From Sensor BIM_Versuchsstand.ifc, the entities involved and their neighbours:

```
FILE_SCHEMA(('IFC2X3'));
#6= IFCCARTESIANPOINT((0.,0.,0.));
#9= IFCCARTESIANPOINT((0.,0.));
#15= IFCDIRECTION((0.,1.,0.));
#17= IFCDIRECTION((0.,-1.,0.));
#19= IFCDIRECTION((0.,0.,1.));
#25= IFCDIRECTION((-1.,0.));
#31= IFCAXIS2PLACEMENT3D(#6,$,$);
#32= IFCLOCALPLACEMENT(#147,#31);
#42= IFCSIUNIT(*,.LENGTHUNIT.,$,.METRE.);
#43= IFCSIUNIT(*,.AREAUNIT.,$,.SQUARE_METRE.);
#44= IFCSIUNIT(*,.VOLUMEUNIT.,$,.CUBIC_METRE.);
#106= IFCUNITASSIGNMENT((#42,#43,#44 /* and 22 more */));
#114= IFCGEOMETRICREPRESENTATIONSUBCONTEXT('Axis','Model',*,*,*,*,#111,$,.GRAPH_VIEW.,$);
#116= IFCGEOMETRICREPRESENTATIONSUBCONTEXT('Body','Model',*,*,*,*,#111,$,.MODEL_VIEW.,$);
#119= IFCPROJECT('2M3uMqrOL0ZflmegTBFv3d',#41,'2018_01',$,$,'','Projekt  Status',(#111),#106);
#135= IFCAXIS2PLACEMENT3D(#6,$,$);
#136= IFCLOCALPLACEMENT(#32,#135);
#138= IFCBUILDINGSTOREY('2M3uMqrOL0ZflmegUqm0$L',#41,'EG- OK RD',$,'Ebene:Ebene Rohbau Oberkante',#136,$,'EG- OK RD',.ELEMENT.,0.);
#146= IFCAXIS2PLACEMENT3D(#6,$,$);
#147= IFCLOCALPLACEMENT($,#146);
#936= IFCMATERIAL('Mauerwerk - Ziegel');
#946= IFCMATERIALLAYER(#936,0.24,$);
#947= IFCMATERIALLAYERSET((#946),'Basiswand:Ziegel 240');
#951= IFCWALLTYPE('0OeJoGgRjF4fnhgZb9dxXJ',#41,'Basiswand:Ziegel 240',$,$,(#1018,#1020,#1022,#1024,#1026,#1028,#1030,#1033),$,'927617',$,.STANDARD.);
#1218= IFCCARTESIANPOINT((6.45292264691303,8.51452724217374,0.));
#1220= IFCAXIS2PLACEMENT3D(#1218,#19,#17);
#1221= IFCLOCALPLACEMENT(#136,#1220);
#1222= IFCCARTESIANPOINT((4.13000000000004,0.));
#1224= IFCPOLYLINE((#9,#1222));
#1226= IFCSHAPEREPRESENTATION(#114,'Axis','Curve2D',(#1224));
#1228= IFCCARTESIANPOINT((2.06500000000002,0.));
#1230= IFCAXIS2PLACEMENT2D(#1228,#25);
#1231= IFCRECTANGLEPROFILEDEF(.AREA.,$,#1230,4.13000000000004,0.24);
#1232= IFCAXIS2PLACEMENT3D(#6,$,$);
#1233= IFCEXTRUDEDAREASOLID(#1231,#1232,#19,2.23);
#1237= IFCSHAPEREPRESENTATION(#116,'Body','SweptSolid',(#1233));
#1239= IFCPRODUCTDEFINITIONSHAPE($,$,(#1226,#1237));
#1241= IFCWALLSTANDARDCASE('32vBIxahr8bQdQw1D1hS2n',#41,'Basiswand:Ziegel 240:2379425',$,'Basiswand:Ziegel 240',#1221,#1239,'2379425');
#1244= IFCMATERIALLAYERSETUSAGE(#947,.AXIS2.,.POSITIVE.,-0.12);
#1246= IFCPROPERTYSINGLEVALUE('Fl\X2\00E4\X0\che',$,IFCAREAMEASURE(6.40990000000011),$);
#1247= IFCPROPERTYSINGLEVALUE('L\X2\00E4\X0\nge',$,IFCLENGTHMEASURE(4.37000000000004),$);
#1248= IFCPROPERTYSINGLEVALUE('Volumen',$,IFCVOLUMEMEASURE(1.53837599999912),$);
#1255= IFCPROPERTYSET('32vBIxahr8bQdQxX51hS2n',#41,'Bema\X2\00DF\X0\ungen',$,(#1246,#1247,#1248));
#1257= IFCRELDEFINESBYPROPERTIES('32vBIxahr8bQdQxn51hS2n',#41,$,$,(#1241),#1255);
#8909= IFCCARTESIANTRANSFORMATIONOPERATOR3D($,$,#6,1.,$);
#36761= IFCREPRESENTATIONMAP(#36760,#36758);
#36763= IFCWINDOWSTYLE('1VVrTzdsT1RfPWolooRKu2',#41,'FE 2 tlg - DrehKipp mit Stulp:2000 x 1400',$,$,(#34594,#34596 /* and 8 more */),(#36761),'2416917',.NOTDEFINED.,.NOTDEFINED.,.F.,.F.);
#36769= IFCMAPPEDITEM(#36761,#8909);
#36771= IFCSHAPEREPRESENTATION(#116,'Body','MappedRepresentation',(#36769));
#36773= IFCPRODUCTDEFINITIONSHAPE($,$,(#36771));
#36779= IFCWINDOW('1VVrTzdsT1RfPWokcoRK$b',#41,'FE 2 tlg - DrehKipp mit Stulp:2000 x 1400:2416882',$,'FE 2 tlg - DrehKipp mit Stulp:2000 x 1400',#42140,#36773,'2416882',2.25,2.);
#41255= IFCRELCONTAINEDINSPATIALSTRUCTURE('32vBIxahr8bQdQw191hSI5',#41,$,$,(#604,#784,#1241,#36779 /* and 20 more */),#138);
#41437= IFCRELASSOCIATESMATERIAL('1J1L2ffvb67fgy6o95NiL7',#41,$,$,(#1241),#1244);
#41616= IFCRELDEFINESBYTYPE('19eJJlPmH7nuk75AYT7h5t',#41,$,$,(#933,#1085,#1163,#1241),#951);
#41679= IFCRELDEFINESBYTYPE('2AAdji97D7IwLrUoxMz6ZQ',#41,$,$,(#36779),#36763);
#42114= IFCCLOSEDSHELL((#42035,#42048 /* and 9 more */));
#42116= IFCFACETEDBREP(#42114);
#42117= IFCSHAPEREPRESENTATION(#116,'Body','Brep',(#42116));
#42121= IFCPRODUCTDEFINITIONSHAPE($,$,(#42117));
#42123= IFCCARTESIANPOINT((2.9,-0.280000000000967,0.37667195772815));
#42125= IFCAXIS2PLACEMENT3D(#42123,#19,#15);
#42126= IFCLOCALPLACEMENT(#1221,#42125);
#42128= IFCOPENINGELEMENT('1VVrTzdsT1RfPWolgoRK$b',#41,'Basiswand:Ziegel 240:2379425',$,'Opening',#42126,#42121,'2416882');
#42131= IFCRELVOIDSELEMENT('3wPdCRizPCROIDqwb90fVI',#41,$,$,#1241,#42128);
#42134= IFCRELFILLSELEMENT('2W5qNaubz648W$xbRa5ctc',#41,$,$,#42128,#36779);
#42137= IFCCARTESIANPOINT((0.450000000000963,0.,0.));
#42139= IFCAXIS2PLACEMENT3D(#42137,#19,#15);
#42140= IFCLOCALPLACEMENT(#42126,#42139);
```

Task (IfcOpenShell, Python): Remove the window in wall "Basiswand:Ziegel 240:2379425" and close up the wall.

```python
import ifcopenshell
import ifcopenshell.api.feature
import ifcopenshell.api.pset
import ifcopenshell.api.root
import ifcopenshell.geom
import ifcopenshell.util.element
import ifcopenshell.util.shape
import ifcopenshell.util.unit

model = ifcopenshell.open("Sensor BIM_Versuchsstand.ifc")
area_scale = ifcopenshell.util.unit.calculate_unit_scale(model, "AREAUNIT")
volume_scale = ifcopenshell.util.unit.calculate_unit_scale(model, "VOLUMEUNIT")
settings = ifcopenshell.geom.settings()


def volume(element):
    """Net volume in cubic metres, openings subtracted."""
    shape = ifcopenshell.geom.create_shape(settings, element)
    return ifcopenshell.util.shape.get_volume(shape.geometry)


window = model.by_id(36779)
opening = window.FillsVoids[0].RelatingOpeningElement
wall = opening.VoidsElements[0].RelatingBuildingElement
before = volume(wall)

ifcopenshell.api.root.remove_product(model, product=window)
ifcopenshell.api.feature.remove_feature(model, feature=opening)

after = volume(wall)
thickness = 0.24  # wall thickness in metres

# Update the wall's stored quantities.
pset = model.by_id(ifcopenshell.util.element.get_pset(wall, "Bemaßungen", should_inherit=False)["id"])
ifcopenshell.api.pset.edit_pset(model, pset=pset, properties={
    "Fläche": model.create_entity("IfcAreaMeasure", after / thickness / area_scale),
    "Volumen": model.create_entity("IfcVolumeMeasure", after / volume_scale),
})

print(f"wall volume {before:.3f} -> {after:.3f} m3")

model.write("Sensor BIM_Versuchsstand_edited.ifc")
```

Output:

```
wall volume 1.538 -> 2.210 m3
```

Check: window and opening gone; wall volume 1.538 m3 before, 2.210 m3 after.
